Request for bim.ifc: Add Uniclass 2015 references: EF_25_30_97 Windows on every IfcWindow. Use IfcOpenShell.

First a look at what the model holds.

```python
import ifcopenshell

model = ifcopenshell.open("bim.ifc")
print(model.schema)
print("classifications:", [c.Name for c in model.by_type("IfcClassification")])
for ifc_class in ("IfcDoor", "IfcRoof", "IfcStair", "IfcWall", "IfcWindow"):
    print(ifc_class, len(model.by_type(ifc_class)))
```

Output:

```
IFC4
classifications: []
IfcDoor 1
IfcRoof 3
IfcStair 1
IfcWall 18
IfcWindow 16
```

```python
import ifcopenshell
import ifcopenshell.api.classification

model = ifcopenshell.open("bim.ifc")

system = ifcopenshell.api.classification.add_classification(model, classification="Uniclass 2015")

codes = {
    "IfcWindow": ("EF_25_30_97", "Windows"),
}
for ifc_class, (code, name) in codes.items():
    products = model.by_type(ifc_class)
    ifcopenshell.api.classification.add_reference(
        model, products=products, classification=system, identification=code, name=name
    )
    print(code, len(products))

model.write("bim_edited.ifc")
```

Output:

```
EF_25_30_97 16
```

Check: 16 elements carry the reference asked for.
